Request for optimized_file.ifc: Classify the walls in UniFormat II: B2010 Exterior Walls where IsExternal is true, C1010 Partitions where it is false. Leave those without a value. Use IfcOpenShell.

First a look at what the model holds.

```python
import ifcopenshell
import ifcopenshell.util.element

model = ifcopenshell.open("optimized_file.ifc")
print(model.schema)
print("classifications:", [c.Name for c in model.by_type("IfcClassification")])
values = [ifcopenshell.util.element.get_pset(e, "Pset_WallCommon", "IsExternal") for e in model.by_type("IfcWall")]
for value in (True, False, None):
    print("IsExternal", value, values.count(value))
```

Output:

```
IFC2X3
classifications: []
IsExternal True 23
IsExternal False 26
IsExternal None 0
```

```python
import ifcopenshell
import ifcopenshell.api.classification
import ifcopenshell.util.element

model = ifcopenshell.open("optimized_file.ifc")

# IFC2X3 requires Source and Edition and has no link from the project to the system.
system = model.create_entity("IfcClassification", Source="ASTM", Edition="E1557", Name="UniFormat II")

walls = model.by_type("IfcWall")
external = {e: ifcopenshell.util.element.get_pset(e, "Pset_WallCommon", "IsExternal") for e in walls}
for flag, code, name in ((True, "B2010", "Exterior Walls"), (False, "C1010", "Partitions")):
    products = [e for e in walls if external[e] is flag]
    ifcopenshell.api.classification.add_reference(
        model, products=products, classification=system, identification=code, name=name
    )
    print(code, len(products))

model.write("optimized_file_rev.ifc")
```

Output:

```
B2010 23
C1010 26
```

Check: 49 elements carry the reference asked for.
